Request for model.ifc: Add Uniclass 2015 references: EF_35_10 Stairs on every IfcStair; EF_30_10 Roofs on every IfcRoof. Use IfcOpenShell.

First a look at what the model holds.

```python
import ifcopenshell

model = ifcopenshell.open("model.ifc")
print(model.schema)
print("classifications:", [c.Name for c in model.by_type("IfcClassification")])
for ifc_class in ("IfcDoor", "IfcRoof", "IfcStair", "IfcWall", "IfcWindow"):
    print(ifc_class, len(model.by_type(ifc_class)))
```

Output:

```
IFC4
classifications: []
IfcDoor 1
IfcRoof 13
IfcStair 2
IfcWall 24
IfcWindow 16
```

```python
import ifcopenshell
import ifcopenshell.api.classification

model = ifcopenshell.open("model.ifc")

system = ifcopenshell.api.classification.add_classification(model, classification="Uniclass 2015")

codes = {
    "IfcStair": ("EF_35_10", "Stairs"),
    "IfcRoof": ("EF_30_10", "Roofs"),
}
for ifc_class, (code, name) in codes.items():
    products = model.by_type(ifc_class)
    ifcopenshell.api.classification.add_reference(
        model, products=products, classification=system, identification=code, name=name
    )
    print(code, len(products))

model.write("model_updated.ifc")
```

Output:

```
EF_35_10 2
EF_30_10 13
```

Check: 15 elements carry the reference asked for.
